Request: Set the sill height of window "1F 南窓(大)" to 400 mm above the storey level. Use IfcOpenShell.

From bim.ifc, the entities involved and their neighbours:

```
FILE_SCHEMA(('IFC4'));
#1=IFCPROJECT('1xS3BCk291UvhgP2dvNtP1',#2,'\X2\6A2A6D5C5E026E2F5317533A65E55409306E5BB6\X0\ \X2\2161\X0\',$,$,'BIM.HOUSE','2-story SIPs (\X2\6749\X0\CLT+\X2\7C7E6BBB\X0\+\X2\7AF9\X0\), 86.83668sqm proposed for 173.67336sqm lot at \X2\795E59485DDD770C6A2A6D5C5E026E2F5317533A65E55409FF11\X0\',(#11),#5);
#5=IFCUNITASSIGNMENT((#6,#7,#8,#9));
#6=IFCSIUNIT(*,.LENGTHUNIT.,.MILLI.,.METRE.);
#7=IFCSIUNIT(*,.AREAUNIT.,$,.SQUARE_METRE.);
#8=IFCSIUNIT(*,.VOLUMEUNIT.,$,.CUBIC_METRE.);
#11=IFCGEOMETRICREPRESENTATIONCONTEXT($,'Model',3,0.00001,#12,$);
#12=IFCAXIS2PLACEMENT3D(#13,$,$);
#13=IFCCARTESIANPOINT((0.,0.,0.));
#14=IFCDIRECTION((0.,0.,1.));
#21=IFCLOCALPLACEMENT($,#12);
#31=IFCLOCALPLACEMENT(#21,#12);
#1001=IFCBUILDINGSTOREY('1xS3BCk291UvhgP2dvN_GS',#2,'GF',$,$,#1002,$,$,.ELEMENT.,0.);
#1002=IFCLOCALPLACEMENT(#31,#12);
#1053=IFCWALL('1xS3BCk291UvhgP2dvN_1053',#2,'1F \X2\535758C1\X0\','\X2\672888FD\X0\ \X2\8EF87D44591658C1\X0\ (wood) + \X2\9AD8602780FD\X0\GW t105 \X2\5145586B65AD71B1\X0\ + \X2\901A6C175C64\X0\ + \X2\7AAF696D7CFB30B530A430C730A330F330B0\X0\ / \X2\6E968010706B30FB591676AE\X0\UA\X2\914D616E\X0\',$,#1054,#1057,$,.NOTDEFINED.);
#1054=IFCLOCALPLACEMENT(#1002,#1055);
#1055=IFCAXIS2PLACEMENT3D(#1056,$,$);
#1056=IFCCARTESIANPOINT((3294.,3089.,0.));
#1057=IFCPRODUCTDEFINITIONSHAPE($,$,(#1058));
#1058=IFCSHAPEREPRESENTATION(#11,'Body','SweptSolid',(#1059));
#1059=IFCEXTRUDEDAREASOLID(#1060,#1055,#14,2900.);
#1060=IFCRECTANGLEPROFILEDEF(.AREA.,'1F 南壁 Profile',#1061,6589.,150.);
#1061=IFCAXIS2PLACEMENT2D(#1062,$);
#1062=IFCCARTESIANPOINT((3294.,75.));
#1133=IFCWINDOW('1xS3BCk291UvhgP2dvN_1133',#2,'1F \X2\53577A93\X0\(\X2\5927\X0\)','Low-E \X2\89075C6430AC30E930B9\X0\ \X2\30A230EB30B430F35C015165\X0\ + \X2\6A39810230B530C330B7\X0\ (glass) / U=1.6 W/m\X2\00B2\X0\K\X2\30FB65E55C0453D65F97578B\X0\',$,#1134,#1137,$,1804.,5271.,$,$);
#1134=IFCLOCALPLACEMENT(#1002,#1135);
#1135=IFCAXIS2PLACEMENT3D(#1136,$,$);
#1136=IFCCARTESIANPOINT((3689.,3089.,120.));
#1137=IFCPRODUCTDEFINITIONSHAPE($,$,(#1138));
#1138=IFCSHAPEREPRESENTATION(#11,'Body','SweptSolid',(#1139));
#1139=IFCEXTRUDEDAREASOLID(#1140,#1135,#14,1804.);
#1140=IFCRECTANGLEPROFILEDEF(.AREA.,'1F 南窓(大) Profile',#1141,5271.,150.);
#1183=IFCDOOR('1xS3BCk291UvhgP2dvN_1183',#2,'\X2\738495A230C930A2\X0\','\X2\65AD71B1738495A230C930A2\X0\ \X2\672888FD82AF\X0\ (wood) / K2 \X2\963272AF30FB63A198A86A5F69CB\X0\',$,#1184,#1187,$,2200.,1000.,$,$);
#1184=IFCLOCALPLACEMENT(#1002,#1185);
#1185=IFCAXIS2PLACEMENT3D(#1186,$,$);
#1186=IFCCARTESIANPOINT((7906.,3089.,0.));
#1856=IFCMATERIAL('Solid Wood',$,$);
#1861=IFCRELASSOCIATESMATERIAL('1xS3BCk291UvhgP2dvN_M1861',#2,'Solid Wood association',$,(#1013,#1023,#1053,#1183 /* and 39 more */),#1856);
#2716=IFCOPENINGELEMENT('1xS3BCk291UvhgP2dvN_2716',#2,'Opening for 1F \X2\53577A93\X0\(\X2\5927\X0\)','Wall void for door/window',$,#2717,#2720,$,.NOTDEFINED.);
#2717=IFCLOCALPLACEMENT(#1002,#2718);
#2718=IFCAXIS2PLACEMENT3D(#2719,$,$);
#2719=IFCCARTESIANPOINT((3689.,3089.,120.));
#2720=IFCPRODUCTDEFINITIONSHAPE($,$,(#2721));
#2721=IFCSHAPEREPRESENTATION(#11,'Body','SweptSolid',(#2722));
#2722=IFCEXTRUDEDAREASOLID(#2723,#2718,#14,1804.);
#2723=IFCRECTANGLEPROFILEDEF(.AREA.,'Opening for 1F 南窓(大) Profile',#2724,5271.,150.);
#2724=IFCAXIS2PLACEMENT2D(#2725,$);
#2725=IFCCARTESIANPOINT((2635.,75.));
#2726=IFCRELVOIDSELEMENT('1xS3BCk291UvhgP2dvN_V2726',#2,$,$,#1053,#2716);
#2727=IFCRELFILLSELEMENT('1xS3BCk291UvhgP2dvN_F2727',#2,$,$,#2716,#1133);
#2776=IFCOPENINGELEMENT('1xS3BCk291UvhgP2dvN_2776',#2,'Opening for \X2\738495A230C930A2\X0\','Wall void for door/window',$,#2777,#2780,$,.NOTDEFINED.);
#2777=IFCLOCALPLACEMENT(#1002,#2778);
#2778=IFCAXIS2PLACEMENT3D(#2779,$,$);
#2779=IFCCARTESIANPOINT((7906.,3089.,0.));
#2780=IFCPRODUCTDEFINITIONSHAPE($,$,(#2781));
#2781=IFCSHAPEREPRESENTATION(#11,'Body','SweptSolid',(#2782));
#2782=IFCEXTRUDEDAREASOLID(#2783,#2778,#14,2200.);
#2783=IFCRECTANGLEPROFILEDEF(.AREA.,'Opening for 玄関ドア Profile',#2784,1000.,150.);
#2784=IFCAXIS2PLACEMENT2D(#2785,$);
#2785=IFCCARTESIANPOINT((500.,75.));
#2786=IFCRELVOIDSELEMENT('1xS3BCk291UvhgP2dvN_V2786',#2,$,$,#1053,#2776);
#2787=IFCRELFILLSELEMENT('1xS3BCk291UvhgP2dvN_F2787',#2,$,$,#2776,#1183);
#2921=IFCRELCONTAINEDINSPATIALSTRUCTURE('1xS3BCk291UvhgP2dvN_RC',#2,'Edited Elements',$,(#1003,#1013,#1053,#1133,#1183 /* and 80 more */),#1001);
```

```python
import numpy as np
import ifcopenshell
import ifcopenshell.api.geometry
import ifcopenshell.geom
import ifcopenshell.util.element
import ifcopenshell.util.placement
import ifcopenshell.util.shape
import ifcopenshell.util.unit

model = ifcopenshell.open("bim.ifc")
unit_scale = ifcopenshell.util.unit.calculate_unit_scale(model)

window = model.by_guid("1xS3BCk291UvhgP2dvN_1133")
opening = window.FillsVoids[0].RelatingOpeningElement
storey = ifcopenshell.util.element.get_container(window, ifc_class="IfcBuildingStorey")
level = ifcopenshell.util.placement.get_local_placement(storey.ObjectPlacement)[2, 3]

# The opening's origin need not be at the sill, so measure its lowest point.
shape = ifcopenshell.geom.create_shape(ifcopenshell.geom.settings(), opening)
bottom = ifcopenshell.util.shape.get_shape_bottom_elevation(shape, shape.geometry) / unit_scale
dz = level + 0.4 / unit_scale - bottom

shift = np.array([0.0, 0.0, dz])
# The window is not placed relative to its opening, so move both.
for product in (opening, window):
    matrix = ifcopenshell.util.placement.get_local_placement(product.ObjectPlacement)
    matrix[:3, 3] += shift
    ifcopenshell.api.geometry.edit_object_placement(model, product=product, matrix=matrix, is_si=False)

print(f"moved by {dz * unit_scale:+.3f} m")

model.write("bim_rev.ifc")
```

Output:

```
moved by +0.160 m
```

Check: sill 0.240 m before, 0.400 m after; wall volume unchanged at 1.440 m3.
